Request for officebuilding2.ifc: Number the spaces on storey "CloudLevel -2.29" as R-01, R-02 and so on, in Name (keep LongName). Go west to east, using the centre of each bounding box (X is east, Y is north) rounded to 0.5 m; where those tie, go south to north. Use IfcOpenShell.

First a look at what the model holds.

```python
import ifcopenshell
import ifcopenshell.util.element
import ifcopenshell.util.placement

model = ifcopenshell.open("officebuilding2.ifc")
print(model.schema)
storey = next(s for s in model.by_type("IfcBuildingStorey") if s.Name == "CloudLevel -2.29")
spaces = [e for e in ifcopenshell.util.element.get_decomposition(storey) if e.is_a("IfcSpace")]
for e in sorted(spaces, key=lambda e: e.id()):
    origin = ifcopenshell.util.placement.get_local_placement(e.ObjectPlacement)[:3, 3]
    print(e.id(), e.Name, e.LongName, origin.round(2) + 0.0, sep=" | ")
```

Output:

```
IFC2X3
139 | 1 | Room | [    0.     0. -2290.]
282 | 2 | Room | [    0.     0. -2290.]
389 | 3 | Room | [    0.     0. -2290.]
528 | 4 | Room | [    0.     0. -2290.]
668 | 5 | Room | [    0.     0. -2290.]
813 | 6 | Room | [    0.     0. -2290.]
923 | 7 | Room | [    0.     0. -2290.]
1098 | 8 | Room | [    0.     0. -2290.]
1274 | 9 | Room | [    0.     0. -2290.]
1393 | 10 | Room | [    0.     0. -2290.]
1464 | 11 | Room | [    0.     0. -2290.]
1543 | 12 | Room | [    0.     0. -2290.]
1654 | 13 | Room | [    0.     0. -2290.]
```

```python
import ifcopenshell
import ifcopenshell.geom
import ifcopenshell.util.element
import ifcopenshell.util.shape

model = ifcopenshell.open("officebuilding2.ifc")
settings = ifcopenshell.geom.settings()
settings.set("use-world-coords", True)


def centre(element):
    shape = ifcopenshell.geom.create_shape(settings, element)
    return ifcopenshell.util.shape.get_bbox_centroid(shape.geometry)


storey = next(s for s in model.by_type("IfcBuildingStorey") if s.Name == "CloudLevel -2.29")
spaces = [e for e in ifcopenshell.util.element.get_decomposition(storey) if e.is_a("IfcSpace")]

# Insertion points can sit at a corner or the storey origin, so sort by the geometry (in metres).
centres = {e: centre(e) for e in spaces}
spaces.sort(key=lambda e: (round(centres[e][0] / 0.5), centres[e][1]))

for i, e in enumerate(spaces, start=1):
    number = f"R-{i:02d}"
    e.Name = number
    print(e.id(), number)

model.write("officebuilding2_v2.ifc")
```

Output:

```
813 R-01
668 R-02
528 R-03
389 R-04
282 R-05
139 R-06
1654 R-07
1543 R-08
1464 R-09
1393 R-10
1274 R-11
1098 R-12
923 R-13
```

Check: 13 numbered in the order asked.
